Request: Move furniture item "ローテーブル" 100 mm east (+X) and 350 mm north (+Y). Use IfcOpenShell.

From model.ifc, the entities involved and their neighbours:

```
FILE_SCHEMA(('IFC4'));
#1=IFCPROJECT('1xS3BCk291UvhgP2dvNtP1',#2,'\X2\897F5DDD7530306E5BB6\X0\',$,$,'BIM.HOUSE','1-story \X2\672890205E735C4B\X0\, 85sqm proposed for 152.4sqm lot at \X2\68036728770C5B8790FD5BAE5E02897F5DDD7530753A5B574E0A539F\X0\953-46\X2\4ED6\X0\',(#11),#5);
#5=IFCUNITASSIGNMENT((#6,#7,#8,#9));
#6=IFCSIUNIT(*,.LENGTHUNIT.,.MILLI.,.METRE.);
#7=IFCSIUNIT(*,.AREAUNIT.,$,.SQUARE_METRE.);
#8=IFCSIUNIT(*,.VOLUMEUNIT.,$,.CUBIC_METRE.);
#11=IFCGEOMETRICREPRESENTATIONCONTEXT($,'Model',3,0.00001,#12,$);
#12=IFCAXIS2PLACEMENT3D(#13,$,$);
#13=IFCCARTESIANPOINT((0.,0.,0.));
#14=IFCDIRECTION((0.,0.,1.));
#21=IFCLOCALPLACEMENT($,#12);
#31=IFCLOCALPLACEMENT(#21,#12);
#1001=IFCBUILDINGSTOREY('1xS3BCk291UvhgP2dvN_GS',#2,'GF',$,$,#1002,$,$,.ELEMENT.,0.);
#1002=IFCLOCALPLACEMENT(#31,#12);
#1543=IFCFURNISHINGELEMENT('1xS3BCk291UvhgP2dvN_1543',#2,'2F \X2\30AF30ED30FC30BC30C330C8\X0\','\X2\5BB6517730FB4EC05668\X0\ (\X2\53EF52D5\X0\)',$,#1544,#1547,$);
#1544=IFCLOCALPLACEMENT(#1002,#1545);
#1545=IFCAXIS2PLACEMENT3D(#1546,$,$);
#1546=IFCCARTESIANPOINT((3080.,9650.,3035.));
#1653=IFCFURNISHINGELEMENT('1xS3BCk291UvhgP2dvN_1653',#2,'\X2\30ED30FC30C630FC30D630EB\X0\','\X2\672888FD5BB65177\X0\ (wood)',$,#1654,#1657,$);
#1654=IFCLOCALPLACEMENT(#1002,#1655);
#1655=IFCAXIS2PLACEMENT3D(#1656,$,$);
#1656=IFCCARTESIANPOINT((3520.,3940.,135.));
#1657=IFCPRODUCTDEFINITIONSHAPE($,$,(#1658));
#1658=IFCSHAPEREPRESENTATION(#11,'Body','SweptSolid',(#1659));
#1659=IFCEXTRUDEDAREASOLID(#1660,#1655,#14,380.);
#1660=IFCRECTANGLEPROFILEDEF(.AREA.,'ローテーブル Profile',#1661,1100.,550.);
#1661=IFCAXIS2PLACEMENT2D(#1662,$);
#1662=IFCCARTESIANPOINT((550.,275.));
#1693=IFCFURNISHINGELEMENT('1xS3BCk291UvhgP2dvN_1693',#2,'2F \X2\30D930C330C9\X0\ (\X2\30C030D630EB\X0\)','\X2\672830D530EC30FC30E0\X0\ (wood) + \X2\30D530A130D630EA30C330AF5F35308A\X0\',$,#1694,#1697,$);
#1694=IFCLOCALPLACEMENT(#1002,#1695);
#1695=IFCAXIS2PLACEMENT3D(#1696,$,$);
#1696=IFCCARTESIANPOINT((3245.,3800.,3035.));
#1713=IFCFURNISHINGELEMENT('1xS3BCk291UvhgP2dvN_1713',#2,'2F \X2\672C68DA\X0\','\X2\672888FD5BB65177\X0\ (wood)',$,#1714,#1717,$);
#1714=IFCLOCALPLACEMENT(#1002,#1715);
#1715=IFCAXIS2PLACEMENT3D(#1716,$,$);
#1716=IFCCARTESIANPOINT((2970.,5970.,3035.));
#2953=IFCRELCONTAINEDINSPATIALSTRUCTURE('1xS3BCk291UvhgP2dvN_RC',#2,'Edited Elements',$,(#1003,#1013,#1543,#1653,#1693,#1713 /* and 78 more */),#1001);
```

```python
import ifcopenshell
import ifcopenshell.api.geometry
import ifcopenshell.util.placement

model = ifcopenshell.open("model.ifc")

item = model.by_guid("1xS3BCk291UvhgP2dvN_1653")
matrix = ifcopenshell.util.placement.get_local_placement(item.ObjectPlacement)
matrix[0, 3] += 100.0
matrix[1, 3] += 350.0
ifcopenshell.api.geometry.edit_object_placement(model, product=item, matrix=matrix, is_si=False)

print(ifcopenshell.util.placement.get_local_placement(item.ObjectPlacement).round(3) + 0.0)

model.write("model_v2.ifc")
```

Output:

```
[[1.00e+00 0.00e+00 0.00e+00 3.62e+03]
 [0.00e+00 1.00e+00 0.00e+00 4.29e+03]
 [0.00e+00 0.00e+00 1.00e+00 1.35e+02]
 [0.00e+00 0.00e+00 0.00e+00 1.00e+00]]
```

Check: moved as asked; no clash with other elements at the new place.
